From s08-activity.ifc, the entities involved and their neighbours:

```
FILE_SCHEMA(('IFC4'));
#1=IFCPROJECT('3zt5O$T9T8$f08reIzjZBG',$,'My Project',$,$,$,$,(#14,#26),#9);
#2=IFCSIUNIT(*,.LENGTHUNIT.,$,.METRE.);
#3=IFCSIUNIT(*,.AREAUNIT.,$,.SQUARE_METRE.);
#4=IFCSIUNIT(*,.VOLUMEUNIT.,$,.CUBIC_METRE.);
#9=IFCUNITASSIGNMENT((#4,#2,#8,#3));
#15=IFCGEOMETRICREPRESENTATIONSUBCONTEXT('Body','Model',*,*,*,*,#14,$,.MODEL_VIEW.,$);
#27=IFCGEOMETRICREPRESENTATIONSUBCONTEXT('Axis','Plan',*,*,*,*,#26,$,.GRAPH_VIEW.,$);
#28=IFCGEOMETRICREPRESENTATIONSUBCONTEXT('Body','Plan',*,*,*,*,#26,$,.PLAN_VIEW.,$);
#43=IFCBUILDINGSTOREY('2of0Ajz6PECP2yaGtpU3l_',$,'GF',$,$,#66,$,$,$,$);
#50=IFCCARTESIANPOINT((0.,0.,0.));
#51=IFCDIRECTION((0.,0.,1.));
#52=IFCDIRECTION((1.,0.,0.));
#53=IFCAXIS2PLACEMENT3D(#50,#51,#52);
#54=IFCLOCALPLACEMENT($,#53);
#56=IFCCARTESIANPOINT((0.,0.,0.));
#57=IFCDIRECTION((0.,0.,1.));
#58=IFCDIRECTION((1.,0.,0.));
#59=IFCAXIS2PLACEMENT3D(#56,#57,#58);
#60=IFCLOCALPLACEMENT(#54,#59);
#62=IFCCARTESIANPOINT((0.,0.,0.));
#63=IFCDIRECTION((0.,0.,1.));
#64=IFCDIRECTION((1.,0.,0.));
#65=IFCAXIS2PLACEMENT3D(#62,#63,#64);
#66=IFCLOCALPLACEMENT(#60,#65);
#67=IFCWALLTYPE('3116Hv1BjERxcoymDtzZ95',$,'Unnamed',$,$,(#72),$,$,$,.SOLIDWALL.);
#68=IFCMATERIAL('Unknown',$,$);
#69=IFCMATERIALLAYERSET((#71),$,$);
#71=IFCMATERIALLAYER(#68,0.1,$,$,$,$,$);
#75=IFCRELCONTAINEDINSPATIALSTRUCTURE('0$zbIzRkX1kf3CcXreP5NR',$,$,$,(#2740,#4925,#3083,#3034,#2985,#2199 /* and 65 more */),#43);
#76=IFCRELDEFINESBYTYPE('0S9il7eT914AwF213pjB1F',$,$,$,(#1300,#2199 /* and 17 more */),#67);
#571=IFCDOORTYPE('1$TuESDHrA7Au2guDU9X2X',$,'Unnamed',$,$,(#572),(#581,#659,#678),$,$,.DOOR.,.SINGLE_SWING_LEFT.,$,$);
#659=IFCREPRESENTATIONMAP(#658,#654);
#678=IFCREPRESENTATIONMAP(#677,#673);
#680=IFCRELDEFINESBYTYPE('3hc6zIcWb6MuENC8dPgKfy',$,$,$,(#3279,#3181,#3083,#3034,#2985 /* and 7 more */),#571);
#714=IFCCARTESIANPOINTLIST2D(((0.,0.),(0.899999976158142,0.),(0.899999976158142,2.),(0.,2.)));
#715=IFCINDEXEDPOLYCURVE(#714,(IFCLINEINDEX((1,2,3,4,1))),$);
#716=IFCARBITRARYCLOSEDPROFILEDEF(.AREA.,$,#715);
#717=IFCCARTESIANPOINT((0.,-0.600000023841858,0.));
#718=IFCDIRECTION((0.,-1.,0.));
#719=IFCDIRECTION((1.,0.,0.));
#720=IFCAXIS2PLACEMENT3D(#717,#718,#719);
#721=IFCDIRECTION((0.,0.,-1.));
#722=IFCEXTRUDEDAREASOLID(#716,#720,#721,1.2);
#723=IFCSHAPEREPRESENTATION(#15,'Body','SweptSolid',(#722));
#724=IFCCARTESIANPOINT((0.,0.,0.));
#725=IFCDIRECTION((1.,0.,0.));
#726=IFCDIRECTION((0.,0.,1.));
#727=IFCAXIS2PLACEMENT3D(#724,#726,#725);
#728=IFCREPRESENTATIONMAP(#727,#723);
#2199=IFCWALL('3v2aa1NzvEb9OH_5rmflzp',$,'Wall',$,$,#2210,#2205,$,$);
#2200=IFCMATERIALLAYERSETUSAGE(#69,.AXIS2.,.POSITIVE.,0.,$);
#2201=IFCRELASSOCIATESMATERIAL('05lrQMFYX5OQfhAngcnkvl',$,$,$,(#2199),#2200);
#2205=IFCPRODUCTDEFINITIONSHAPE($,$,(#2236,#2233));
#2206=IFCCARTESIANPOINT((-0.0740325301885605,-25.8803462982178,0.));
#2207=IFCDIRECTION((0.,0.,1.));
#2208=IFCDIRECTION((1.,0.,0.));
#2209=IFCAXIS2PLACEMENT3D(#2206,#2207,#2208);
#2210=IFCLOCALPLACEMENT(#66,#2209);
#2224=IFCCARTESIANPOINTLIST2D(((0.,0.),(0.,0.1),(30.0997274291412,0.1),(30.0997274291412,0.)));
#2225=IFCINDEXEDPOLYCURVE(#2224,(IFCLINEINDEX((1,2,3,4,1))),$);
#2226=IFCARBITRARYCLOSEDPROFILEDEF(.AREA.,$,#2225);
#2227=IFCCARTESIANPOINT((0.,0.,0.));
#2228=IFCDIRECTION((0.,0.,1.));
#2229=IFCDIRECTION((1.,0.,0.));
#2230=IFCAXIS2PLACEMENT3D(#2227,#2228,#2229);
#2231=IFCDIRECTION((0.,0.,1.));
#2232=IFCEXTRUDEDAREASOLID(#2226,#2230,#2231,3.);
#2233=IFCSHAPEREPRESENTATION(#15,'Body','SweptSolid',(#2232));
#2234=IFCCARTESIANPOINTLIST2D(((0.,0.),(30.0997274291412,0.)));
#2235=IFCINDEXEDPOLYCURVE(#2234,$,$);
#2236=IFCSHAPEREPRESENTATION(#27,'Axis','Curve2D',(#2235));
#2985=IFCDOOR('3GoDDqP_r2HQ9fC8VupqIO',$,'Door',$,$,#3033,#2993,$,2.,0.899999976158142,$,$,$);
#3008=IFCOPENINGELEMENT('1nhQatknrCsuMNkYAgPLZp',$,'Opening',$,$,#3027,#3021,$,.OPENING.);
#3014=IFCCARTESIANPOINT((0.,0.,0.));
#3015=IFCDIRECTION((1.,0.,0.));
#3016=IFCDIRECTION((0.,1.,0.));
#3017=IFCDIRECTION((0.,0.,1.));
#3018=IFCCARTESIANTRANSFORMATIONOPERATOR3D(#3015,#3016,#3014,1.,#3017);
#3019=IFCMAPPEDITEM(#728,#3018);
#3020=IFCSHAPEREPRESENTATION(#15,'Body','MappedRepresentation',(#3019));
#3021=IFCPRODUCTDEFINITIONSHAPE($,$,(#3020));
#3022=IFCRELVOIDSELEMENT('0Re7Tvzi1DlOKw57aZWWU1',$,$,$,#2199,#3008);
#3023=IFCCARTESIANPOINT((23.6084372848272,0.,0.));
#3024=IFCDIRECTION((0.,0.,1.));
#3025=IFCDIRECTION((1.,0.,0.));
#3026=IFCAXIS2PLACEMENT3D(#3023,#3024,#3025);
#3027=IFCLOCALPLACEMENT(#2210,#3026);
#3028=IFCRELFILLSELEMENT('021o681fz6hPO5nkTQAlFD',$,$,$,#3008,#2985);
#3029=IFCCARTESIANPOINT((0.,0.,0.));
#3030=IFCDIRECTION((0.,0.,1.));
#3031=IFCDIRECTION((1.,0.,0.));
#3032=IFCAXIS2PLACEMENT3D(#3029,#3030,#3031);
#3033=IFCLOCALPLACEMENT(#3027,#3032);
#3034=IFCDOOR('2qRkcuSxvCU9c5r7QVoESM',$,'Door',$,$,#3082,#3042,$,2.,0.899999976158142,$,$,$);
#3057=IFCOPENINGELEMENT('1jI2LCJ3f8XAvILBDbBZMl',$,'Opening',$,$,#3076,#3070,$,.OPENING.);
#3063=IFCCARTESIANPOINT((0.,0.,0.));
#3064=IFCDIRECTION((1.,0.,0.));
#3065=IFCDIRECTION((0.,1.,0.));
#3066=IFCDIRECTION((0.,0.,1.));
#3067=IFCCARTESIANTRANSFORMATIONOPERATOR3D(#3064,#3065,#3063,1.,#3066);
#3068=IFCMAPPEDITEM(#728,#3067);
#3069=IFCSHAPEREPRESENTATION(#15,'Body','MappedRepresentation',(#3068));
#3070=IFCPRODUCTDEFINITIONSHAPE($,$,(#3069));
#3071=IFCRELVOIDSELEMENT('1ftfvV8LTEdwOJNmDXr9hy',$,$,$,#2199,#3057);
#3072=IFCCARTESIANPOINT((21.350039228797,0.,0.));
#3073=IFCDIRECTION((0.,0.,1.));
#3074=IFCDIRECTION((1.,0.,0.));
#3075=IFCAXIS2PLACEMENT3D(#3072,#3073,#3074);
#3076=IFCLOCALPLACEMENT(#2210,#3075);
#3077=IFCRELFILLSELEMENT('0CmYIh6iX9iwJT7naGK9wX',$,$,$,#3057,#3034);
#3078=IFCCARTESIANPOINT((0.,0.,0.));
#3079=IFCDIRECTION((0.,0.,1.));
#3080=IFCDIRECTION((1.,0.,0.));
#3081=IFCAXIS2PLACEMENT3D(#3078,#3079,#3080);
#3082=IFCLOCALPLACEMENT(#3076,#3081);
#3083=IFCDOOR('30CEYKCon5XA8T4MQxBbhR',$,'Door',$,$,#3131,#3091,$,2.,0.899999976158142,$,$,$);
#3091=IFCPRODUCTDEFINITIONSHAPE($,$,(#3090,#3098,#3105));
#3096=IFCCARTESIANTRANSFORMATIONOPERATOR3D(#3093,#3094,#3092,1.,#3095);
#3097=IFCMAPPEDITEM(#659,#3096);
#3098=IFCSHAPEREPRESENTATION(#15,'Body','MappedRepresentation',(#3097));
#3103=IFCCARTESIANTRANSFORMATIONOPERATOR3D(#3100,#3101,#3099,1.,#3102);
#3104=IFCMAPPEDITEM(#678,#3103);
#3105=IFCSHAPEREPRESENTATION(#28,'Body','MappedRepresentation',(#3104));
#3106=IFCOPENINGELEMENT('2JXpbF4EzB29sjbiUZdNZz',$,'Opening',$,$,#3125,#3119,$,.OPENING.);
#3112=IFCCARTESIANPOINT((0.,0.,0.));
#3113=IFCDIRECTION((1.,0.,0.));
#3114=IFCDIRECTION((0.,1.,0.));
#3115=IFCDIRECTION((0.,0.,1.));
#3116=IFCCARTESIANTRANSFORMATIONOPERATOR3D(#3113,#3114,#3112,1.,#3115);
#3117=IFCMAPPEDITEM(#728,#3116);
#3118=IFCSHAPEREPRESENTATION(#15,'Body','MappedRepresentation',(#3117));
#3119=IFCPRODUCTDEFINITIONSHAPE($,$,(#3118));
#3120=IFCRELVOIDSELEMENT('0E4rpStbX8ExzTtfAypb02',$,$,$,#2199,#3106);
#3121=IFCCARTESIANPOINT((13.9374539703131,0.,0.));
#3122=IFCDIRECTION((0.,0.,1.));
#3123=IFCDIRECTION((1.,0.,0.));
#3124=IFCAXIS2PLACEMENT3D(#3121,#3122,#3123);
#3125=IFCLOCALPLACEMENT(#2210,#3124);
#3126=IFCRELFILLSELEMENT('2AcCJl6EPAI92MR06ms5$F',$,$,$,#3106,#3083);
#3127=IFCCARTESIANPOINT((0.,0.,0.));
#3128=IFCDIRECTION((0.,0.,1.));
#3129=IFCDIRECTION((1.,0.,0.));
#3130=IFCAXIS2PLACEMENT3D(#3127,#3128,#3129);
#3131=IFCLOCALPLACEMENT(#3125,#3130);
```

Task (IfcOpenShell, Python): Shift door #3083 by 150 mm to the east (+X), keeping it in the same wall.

```python
import ifcopenshell
import ifcopenshell.api.geometry
import ifcopenshell.util.placement
import ifcopenshell.util.unit

model = ifcopenshell.open("s08-activity.ifc")
unit_scale = ifcopenshell.util.unit.calculate_unit_scale(model)

door = model.by_guid("30CEYKCon5XA8T4MQxBbhR")
opening = door.FillsVoids[0].RelatingOpeningElement
wall = opening.VoidsElements[0].RelatingBuildingElement

wall_matrix = ifcopenshell.util.placement.get_local_placement(wall.ObjectPlacement)
shift = wall_matrix[:3, 0] * 0.15 / unit_scale
before = ifcopenshell.util.placement.get_local_placement(door.ObjectPlacement)[:3, 3].copy()

# The door is placed relative to its opening, so it follows when the opening moves.
matrix = ifcopenshell.util.placement.get_local_placement(opening.ObjectPlacement)
matrix[:3, 3] += shift
ifcopenshell.api.geometry.edit_object_placement(
    model, product=opening, matrix=matrix, is_si=False, should_transform_children=True
)

after = ifcopenshell.util.placement.get_local_placement(door.ObjectPlacement)[:3, 3]
print("door moved by", (after - before).round(3) + 0.0)

model.write("s08-activity_v2.ifc")
```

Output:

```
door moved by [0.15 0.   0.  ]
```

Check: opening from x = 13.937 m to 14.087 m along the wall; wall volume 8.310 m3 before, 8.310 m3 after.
